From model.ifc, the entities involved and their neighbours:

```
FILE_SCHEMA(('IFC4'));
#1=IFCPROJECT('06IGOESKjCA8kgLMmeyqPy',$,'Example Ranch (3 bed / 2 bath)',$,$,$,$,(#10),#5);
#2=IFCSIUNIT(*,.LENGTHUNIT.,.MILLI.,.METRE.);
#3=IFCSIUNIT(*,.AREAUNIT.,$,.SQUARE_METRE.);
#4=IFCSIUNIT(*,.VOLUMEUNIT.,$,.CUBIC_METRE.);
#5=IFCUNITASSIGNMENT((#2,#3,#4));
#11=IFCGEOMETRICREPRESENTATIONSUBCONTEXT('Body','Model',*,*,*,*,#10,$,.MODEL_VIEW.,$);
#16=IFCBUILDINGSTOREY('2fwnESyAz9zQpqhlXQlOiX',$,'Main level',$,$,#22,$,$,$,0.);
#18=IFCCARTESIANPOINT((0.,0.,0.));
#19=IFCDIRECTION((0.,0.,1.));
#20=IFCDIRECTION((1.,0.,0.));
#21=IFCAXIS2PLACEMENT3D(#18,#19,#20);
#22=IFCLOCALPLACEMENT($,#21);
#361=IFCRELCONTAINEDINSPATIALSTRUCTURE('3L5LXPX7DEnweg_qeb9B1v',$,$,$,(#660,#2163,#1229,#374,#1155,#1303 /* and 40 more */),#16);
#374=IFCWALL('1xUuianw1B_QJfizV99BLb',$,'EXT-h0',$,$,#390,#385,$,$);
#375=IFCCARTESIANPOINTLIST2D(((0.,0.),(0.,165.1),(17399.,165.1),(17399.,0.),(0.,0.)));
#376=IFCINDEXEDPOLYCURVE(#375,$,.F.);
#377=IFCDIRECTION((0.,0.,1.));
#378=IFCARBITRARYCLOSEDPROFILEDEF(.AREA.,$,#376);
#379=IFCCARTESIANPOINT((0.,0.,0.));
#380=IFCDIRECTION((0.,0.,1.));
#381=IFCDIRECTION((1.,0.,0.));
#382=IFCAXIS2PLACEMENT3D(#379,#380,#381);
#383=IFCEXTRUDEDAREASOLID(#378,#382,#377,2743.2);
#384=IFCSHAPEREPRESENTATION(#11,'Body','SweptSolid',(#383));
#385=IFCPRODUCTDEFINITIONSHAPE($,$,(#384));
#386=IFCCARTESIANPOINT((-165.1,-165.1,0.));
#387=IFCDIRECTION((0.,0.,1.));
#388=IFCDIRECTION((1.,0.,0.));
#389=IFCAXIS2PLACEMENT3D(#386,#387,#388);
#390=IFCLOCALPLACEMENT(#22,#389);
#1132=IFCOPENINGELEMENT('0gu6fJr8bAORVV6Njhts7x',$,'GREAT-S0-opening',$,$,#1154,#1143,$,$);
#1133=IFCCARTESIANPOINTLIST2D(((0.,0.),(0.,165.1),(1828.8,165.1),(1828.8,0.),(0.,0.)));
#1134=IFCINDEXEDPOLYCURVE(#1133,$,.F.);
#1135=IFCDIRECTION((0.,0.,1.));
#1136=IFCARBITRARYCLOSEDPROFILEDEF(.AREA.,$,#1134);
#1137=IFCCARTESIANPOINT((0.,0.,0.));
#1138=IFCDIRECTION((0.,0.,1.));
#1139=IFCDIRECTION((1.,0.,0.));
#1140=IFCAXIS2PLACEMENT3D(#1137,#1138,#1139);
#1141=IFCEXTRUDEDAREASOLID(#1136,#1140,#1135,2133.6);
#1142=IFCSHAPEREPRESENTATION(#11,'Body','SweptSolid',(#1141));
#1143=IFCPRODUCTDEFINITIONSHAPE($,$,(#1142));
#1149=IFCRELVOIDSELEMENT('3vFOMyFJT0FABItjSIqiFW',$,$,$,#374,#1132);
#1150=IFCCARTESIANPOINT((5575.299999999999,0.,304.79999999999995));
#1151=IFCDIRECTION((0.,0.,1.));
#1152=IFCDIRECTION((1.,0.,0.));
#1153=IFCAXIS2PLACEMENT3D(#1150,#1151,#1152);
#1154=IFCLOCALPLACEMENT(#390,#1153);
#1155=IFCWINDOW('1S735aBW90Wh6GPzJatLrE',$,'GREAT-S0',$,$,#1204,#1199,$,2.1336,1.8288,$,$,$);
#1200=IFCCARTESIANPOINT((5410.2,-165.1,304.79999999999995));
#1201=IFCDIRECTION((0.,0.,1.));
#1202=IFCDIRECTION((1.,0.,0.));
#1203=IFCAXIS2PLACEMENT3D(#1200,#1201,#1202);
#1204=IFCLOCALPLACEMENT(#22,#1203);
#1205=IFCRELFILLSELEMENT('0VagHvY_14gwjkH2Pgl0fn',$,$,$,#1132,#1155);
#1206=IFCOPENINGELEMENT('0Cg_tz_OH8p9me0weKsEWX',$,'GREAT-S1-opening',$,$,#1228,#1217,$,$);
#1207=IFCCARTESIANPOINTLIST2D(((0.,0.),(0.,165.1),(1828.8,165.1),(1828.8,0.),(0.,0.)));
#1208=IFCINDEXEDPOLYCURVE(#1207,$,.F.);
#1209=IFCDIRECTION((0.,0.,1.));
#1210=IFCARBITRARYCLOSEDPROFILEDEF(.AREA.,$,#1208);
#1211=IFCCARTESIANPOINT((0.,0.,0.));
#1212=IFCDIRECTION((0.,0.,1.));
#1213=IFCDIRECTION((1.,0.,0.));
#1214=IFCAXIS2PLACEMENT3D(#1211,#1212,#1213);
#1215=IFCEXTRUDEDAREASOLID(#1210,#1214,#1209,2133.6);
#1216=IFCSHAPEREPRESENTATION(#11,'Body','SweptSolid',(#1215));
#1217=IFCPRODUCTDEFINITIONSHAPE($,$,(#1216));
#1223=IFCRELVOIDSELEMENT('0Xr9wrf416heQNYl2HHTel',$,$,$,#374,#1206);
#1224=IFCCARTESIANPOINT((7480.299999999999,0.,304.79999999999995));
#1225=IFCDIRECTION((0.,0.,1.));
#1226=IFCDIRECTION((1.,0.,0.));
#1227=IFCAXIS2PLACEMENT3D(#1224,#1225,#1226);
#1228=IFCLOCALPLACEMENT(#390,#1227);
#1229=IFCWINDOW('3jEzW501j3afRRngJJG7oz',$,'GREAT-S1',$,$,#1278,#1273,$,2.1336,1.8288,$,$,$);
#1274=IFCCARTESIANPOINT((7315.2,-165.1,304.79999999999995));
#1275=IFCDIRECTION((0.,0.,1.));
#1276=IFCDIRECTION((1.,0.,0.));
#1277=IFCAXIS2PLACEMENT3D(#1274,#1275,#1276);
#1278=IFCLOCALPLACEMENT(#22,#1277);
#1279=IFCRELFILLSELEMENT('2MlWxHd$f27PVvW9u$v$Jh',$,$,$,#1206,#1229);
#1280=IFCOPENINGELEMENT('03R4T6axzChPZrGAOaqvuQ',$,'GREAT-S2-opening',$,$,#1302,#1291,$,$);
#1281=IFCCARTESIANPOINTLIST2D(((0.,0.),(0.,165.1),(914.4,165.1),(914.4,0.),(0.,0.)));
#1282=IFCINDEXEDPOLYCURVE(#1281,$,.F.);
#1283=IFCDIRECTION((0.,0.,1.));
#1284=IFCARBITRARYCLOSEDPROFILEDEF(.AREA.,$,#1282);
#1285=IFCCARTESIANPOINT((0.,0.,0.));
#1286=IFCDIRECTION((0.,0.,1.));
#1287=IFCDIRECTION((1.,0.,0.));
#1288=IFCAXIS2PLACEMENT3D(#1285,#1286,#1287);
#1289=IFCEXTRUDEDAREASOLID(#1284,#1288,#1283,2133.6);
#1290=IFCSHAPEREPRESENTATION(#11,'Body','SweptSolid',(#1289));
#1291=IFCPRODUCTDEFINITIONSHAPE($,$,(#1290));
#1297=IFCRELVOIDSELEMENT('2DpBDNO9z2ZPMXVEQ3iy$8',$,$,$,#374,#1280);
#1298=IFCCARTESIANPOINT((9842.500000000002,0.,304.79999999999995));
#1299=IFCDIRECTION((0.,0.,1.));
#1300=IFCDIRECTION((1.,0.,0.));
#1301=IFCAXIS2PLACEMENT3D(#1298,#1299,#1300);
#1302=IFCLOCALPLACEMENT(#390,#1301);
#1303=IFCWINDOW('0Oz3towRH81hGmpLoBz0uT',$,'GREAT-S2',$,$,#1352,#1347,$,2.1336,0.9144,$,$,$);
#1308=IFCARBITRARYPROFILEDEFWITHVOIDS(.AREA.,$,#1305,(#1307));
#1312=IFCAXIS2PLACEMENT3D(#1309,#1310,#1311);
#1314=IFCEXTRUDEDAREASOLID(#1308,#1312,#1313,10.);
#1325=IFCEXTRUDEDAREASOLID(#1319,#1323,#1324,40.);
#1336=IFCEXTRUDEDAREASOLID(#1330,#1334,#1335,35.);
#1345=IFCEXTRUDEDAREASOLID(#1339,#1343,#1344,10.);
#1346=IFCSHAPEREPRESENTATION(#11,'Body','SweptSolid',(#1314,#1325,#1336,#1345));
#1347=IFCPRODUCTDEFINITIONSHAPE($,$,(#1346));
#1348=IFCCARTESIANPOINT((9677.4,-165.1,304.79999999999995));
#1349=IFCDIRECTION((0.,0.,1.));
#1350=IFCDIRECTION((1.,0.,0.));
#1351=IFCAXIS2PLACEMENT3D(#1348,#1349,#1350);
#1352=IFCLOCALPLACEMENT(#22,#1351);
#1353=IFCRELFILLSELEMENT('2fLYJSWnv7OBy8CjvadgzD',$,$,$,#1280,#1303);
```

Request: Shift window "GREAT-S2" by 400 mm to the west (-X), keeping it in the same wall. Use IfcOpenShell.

```python
import ifcopenshell
import ifcopenshell.api.geometry
import ifcopenshell.util.placement

model = ifcopenshell.open("model.ifc")

window = model.by_guid("0Oz3towRH81hGmpLoBz0uT")
opening = window.FillsVoids[0].RelatingOpeningElement
wall = opening.VoidsElements[0].RelatingBuildingElement

wall_matrix = ifcopenshell.util.placement.get_local_placement(wall.ObjectPlacement)
shift = wall_matrix[:3, 0] * -400.0
before = ifcopenshell.util.placement.get_local_placement(window.ObjectPlacement)[:3, 3].copy()

# The window is not placed relative to its opening, so move both.
for product in (opening, window):
    matrix = ifcopenshell.util.placement.get_local_placement(product.ObjectPlacement)
    matrix[:3, 3] += shift
    ifcopenshell.api.geometry.edit_object_placement(model, product=product, matrix=matrix, is_si=False)

after = ifcopenshell.util.placement.get_local_placement(window.ObjectPlacement)[:3, 3]
print("window moved by", (after - before).round(3) + 0.0)

model.write("model_updated.ifc")
```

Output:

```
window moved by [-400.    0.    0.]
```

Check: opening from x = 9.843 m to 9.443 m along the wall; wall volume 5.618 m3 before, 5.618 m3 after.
